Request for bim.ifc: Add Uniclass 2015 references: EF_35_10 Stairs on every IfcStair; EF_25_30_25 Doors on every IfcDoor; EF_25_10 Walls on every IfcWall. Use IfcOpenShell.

First a look at what the model holds.

```python
import ifcopenshell

model = ifcopenshell.open("bim.ifc")
print(model.schema)
print("classifications:", [c.Name for c in model.by_type("IfcClassification")])
for ifc_class in ("IfcDoor", "IfcRoof", "IfcStair", "IfcWall", "IfcWindow"):
    print(ifc_class, len(model.by_type(ifc_class)))
```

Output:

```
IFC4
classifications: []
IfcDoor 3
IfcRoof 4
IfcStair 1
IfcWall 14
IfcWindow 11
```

```python
import ifcopenshell
import ifcopenshell.api.classification

model = ifcopenshell.open("bim.ifc")

system = ifcopenshell.api.classification.add_classification(model, classification="Uniclass 2015")

codes = {
    "IfcStair": ("EF_35_10", "Stairs"),
    "IfcDoor": ("EF_25_30_25", "Doors"),
    "IfcWall": ("EF_25_10", "Walls"),
}
for ifc_class, (code, name) in codes.items():
    products = model.by_type(ifc_class)
    ifcopenshell.api.classification.add_reference(
        model, products=products, classification=system, identification=code, name=name
    )
    print(code, len(products))

model.write("bim_v2.ifc")
```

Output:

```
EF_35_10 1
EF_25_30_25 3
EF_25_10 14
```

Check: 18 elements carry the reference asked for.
